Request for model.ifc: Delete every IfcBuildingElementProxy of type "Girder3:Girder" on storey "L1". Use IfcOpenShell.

First a look at what the model holds.

```python
import ifcopenshell
import ifcopenshell.util.element

model = ifcopenshell.open("model.ifc")
print(model.schema)
storey = next(s for s in model.by_type("IfcBuildingStorey") if s.Name == "L1")
proxies = [e for e in ifcopenshell.util.element.get_decomposition(storey) if e.is_a("IfcBuildingElementProxy")]
seen = {}
for e in proxies:
    element_type = ifcopenshell.util.element.get_type(e)
    name = element_type.Name if element_type not in (None, e) else None
    seen[name] = seen.get(name, 0) + 1
for name, count in sorted(seen.items(), key=str):
    print(count, "x", name)
```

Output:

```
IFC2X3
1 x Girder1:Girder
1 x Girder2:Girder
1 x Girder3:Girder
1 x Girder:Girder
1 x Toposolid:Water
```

```python
import ifcopenshell
import ifcopenshell.api.root
import ifcopenshell.util.element

model = ifcopenshell.open("model.ifc")

storey = next(s for s in model.by_type("IfcBuildingStorey") if s.Name == "L1")
proxies = [e for e in ifcopenshell.util.element.get_decomposition(storey) if e.is_a("IfcBuildingElementProxy")]
targets = [e for e in proxies if (t := ifcopenshell.util.element.get_type(e)) not in (None, e) and t.Name == "Girder3:Girder"]

for e in targets:
    ifcopenshell.api.root.remove_product(model, product=e)
print(len(targets), "removed")

model.write("model_v2.ifc")
```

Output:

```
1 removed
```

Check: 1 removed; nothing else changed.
